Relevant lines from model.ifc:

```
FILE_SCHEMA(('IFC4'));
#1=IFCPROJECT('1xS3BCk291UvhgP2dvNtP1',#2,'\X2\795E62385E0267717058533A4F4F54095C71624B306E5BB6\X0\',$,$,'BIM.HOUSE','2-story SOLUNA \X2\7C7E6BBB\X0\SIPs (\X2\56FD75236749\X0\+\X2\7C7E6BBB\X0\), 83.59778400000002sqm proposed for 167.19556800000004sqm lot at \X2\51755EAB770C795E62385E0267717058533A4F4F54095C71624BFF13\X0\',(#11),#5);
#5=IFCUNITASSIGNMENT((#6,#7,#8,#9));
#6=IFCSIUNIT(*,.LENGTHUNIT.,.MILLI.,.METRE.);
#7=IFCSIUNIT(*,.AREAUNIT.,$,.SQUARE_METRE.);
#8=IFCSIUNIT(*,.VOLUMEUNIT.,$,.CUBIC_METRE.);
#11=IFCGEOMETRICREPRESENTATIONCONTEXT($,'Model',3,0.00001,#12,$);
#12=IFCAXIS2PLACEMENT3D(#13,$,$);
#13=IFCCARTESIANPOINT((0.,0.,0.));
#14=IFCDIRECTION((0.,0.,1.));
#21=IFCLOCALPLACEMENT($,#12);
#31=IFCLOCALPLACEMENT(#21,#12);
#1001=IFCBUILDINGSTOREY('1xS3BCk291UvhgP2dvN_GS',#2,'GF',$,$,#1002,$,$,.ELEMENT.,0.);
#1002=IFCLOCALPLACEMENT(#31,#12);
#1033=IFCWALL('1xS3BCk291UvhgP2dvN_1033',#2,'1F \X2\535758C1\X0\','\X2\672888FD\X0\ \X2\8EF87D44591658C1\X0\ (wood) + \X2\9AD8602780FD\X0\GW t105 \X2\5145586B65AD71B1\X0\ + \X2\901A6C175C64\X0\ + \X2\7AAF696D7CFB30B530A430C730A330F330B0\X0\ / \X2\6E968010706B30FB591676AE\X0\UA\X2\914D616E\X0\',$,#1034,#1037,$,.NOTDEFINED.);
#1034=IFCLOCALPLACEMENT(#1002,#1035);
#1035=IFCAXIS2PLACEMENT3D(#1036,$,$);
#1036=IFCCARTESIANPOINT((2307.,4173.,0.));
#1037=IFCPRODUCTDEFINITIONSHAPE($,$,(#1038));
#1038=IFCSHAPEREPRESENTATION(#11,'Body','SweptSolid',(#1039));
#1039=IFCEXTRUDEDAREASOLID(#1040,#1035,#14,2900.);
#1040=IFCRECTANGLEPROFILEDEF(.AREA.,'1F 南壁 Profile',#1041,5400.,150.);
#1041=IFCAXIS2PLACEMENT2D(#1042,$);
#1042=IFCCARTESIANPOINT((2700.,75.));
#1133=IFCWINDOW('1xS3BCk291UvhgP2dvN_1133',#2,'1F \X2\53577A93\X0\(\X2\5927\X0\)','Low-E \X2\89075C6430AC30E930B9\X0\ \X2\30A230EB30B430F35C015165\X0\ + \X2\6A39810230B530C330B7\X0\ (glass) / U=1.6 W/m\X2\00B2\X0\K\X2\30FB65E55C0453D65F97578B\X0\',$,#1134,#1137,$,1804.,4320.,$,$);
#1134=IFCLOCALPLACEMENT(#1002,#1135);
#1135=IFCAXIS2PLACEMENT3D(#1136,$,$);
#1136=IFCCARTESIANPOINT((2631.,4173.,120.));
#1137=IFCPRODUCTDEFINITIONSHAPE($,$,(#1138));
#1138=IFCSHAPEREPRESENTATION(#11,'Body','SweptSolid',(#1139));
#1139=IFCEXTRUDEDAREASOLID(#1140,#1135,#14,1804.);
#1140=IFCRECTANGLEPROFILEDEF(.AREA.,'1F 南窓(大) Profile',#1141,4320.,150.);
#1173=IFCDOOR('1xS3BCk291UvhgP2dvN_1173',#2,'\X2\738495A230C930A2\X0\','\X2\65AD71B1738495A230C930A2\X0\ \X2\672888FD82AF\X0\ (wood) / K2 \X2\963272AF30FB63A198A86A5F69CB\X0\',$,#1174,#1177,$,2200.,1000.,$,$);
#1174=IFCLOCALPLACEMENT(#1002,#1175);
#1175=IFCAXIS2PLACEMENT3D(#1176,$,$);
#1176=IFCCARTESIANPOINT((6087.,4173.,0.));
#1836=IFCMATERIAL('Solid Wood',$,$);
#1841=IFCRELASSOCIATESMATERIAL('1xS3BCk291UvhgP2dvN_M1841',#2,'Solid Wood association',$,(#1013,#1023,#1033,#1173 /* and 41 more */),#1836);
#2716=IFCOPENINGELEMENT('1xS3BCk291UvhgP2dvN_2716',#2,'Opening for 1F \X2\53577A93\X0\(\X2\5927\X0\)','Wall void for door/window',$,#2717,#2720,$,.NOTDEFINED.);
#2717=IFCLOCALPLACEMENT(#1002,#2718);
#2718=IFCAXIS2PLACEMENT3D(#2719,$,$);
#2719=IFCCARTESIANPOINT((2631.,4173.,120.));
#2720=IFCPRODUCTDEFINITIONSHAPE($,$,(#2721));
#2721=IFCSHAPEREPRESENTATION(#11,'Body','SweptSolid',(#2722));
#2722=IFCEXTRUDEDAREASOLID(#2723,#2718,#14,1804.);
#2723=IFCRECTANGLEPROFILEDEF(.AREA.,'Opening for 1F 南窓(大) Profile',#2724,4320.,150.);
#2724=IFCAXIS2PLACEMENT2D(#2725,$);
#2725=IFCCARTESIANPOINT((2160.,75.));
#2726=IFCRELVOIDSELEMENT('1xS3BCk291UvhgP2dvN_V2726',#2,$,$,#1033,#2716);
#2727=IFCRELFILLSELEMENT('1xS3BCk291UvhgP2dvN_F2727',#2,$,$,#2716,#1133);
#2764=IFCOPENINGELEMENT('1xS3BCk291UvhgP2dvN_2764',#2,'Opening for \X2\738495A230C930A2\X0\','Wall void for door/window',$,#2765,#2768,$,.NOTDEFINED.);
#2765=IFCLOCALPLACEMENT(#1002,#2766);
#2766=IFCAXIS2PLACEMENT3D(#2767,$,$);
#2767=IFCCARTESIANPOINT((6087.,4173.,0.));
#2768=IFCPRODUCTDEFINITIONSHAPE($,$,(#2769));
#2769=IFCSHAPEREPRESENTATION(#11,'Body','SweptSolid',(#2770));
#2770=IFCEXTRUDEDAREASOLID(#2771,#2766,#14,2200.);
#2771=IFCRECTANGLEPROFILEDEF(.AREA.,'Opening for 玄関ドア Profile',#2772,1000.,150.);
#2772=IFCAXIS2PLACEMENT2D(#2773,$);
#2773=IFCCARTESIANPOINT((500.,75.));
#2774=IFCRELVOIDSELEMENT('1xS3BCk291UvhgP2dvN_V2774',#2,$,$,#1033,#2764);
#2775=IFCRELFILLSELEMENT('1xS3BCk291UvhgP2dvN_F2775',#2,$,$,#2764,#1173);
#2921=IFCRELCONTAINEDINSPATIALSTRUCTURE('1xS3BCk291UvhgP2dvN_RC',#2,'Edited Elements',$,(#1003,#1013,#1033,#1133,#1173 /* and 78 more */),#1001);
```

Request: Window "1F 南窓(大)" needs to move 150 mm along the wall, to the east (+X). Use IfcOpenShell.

```python
import ifcopenshell
import ifcopenshell.api.geometry
import ifcopenshell.util.placement

model = ifcopenshell.open("model.ifc")

window = model.by_guid("1xS3BCk291UvhgP2dvN_1133")
opening = window.FillsVoids[0].RelatingOpeningElement
wall = opening.VoidsElements[0].RelatingBuildingElement

wall_matrix = ifcopenshell.util.placement.get_local_placement(wall.ObjectPlacement)
shift = wall_matrix[:3, 0] * 150.0
before = ifcopenshell.util.placement.get_local_placement(window.ObjectPlacement)[:3, 3].copy()

# The window is not placed relative to its opening, so move both.
for product in (opening, window):
    matrix = ifcopenshell.util.placement.get_local_placement(product.ObjectPlacement)
    matrix[:3, 3] += shift
    ifcopenshell.api.geometry.edit_object_placement(model, product=product, matrix=matrix, is_si=False)

after = ifcopenshell.util.placement.get_local_placement(window.ObjectPlacement)[:3, 3]
print("window moved by", (after - before).round(3) + 0.0)

model.write("model_rev.ifc")
```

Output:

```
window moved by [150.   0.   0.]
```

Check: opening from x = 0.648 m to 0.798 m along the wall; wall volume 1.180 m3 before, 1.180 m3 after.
